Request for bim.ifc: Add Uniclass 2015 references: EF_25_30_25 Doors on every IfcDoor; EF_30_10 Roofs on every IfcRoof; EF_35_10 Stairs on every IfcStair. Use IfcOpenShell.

First a look at what the model holds.

```python
import ifcopenshell

model = ifcopenshell.open("bim.ifc")
print(model.schema)
print("classifications:", [c.Name for c in model.by_type("IfcClassification")])
for ifc_class in ("IfcDoor", "IfcRoof", "IfcStair", "IfcWall", "IfcWindow"):
    print(ifc_class, len(model.by_type(ifc_class)))
```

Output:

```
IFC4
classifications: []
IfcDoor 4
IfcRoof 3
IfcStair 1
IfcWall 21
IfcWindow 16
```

```python
import ifcopenshell
import ifcopenshell.api.classification

model = ifcopenshell.open("bim.ifc")

system = ifcopenshell.api.classification.add_classification(model, classification="Uniclass 2015")

codes = {
    "IfcDoor": ("EF_25_30_25", "Doors"),
    "IfcRoof": ("EF_30_10", "Roofs"),
    "IfcStair": ("EF_35_10", "Stairs"),
}
for ifc_class, (code, name) in codes.items():
    products = model.by_type(ifc_class)
    ifcopenshell.api.classification.add_reference(
        model, products=products, classification=system, identification=code, name=name
    )
    print(code, len(products))

model.write("bim-out.ifc")
```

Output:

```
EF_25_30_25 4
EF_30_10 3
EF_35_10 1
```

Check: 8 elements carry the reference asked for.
